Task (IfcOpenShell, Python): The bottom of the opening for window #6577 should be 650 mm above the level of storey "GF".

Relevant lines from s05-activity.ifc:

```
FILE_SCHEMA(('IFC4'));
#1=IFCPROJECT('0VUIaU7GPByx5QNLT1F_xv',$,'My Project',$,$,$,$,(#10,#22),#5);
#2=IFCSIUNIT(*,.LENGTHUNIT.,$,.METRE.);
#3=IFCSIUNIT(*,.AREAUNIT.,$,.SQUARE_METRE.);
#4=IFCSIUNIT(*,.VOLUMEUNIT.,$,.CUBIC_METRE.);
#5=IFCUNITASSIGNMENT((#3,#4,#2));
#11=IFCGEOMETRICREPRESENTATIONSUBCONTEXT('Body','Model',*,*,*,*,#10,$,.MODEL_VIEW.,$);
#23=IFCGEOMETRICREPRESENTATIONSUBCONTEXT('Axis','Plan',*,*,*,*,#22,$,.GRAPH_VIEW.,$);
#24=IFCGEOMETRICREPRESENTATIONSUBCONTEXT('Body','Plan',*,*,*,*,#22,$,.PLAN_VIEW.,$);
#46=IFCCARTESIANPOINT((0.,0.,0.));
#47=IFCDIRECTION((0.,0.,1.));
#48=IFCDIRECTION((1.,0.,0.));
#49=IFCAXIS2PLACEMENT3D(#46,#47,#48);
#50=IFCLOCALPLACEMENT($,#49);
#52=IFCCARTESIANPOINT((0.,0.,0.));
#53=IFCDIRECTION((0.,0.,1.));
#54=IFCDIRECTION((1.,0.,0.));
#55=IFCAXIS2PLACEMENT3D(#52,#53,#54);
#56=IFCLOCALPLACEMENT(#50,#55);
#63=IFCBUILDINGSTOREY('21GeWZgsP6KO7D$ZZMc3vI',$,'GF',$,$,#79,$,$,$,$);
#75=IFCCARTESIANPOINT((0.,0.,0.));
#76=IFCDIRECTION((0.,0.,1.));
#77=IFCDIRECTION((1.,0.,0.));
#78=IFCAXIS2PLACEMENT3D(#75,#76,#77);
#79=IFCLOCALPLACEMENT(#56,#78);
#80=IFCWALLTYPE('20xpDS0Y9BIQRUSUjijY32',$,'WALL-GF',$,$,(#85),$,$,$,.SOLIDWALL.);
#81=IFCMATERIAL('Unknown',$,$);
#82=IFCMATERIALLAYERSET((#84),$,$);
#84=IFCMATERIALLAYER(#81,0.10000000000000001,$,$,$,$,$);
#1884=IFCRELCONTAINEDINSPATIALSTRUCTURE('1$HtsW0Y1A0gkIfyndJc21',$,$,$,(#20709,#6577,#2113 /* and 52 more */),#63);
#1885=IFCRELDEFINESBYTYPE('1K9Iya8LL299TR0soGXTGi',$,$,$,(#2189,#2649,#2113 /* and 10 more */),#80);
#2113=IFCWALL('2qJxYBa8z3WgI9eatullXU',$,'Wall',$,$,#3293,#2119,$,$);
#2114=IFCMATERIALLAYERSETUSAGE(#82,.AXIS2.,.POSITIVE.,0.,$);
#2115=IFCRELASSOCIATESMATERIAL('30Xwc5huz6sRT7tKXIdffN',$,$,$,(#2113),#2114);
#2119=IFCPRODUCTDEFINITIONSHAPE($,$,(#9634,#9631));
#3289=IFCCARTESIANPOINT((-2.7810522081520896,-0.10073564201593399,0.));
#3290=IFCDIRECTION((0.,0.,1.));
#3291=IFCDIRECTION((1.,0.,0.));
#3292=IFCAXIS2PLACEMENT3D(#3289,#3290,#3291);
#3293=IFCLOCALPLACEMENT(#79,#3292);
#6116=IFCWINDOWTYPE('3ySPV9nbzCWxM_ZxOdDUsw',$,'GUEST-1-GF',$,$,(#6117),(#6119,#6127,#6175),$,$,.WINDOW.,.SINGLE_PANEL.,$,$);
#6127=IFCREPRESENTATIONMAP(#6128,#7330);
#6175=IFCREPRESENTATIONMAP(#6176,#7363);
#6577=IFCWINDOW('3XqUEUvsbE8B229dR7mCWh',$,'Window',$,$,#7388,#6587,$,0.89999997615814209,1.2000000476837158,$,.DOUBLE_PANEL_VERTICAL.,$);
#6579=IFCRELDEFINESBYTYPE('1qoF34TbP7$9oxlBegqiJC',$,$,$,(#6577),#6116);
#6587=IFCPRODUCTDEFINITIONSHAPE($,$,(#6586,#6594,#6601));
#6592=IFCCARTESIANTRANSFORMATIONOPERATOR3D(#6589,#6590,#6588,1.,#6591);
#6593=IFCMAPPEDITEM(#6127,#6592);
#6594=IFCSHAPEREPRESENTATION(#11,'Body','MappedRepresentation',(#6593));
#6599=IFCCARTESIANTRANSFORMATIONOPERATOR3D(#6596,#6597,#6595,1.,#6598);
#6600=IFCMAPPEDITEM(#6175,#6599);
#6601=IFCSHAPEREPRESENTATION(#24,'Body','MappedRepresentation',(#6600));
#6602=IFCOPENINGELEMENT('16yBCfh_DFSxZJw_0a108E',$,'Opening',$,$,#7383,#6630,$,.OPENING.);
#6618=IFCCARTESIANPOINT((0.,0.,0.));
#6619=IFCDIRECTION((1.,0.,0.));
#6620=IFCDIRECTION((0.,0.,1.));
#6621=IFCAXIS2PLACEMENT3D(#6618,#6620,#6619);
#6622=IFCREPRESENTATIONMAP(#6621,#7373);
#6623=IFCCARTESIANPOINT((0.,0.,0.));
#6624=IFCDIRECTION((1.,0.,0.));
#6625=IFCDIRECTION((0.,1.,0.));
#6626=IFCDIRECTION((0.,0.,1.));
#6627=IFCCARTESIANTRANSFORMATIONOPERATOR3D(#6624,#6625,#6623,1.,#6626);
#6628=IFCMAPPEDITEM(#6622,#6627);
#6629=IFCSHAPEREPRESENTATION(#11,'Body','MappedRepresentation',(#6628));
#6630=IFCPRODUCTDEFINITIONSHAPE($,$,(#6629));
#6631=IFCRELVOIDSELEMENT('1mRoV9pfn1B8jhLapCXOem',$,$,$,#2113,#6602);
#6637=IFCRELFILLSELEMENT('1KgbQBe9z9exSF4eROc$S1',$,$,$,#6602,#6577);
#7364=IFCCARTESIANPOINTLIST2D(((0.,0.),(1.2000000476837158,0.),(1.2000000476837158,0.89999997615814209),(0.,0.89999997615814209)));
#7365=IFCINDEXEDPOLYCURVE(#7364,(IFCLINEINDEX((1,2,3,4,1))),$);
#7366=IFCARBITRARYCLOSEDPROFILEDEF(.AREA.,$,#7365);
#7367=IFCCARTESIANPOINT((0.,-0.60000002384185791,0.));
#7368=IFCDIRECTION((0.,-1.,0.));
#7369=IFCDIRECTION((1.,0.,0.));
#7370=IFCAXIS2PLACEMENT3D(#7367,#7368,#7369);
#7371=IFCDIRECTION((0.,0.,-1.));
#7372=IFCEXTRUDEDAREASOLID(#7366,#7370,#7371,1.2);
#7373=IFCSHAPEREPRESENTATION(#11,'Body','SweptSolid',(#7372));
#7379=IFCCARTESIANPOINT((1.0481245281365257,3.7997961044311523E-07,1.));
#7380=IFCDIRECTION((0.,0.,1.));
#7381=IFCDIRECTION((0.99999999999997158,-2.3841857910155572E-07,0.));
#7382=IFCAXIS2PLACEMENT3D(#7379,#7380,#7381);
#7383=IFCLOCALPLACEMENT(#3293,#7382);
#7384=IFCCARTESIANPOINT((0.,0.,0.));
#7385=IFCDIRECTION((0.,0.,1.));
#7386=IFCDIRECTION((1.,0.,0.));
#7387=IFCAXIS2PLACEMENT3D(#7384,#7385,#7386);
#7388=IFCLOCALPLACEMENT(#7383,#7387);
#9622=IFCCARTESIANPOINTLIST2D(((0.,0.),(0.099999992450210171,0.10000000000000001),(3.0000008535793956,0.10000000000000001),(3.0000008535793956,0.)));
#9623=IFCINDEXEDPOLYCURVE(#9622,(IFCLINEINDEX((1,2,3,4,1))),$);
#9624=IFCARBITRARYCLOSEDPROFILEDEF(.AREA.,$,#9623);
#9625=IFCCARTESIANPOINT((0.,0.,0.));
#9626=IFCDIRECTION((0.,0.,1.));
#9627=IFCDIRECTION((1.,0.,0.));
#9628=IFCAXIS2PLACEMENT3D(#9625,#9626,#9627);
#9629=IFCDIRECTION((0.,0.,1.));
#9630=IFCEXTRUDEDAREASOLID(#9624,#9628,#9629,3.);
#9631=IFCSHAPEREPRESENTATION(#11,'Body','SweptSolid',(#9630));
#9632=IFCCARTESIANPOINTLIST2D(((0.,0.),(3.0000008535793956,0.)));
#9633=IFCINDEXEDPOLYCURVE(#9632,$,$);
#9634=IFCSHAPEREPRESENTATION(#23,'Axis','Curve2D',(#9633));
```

```python
import numpy as np
import ifcopenshell
import ifcopenshell.api.geometry
import ifcopenshell.geom
import ifcopenshell.util.element
import ifcopenshell.util.placement
import ifcopenshell.util.shape
import ifcopenshell.util.unit

model = ifcopenshell.open("s05-activity.ifc")
unit_scale = ifcopenshell.util.unit.calculate_unit_scale(model)

window = model.by_guid("3XqUEUvsbE8B229dR7mCWh")
opening = window.FillsVoids[0].RelatingOpeningElement
storey = ifcopenshell.util.element.get_container(window, ifc_class="IfcBuildingStorey")
level = ifcopenshell.util.placement.get_local_placement(storey.ObjectPlacement)[2, 3]

# The opening's origin need not be at the sill, so measure its lowest point.
shape = ifcopenshell.geom.create_shape(ifcopenshell.geom.settings(), opening)
bottom = ifcopenshell.util.shape.get_shape_bottom_elevation(shape, shape.geometry) / unit_scale
dz = level + 0.65 / unit_scale - bottom

shift = np.array([0.0, 0.0, dz])
# The window is placed relative to its opening, so it follows when the opening moves.
matrix = ifcopenshell.util.placement.get_local_placement(opening.ObjectPlacement)
matrix[:3, 3] += shift
ifcopenshell.api.geometry.edit_object_placement(
    model, product=opening, matrix=matrix, is_si=False, should_transform_children=True
)

print(f"moved by {dz * unit_scale:+.3f} m")

model.write("s05-activity_edited.ifc")
```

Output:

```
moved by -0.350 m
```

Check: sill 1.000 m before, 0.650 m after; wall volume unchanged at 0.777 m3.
